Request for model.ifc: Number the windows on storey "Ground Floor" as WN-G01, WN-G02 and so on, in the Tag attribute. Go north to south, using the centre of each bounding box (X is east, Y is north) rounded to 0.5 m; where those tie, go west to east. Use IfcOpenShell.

First a look at what the model holds.

```python
import ifcopenshell
import ifcopenshell.util.element
import ifcopenshell.util.placement

model = ifcopenshell.open("model.ifc")
print(model.schema)
storey = next(s for s in model.by_type("IfcBuildingStorey") if s.Name == "Ground Floor")
windows = [e for e in ifcopenshell.util.element.get_decomposition(storey) if e.is_a("IfcWindow")]
for e in sorted(windows, key=lambda e: e.id()):
    origin = ifcopenshell.util.placement.get_local_placement(e.ObjectPlacement)[:3, 3]
    print(e.id(), e.Tag, e.Name, origin.round(2) + 0.0, sep=" | ")
```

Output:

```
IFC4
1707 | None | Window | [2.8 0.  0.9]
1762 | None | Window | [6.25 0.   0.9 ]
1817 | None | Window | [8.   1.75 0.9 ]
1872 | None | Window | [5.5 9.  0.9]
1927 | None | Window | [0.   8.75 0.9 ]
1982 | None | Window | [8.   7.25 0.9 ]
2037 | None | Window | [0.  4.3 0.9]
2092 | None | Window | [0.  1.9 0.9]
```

```python
import ifcopenshell
import ifcopenshell.geom
import ifcopenshell.util.element
import ifcopenshell.util.shape

model = ifcopenshell.open("model.ifc")
settings = ifcopenshell.geom.settings()
settings.set("use-world-coords", True)


def centre(element):
    shape = ifcopenshell.geom.create_shape(settings, element)
    return ifcopenshell.util.shape.get_bbox_centroid(shape.geometry)


storey = next(s for s in model.by_type("IfcBuildingStorey") if s.Name == "Ground Floor")
windows = [e for e in ifcopenshell.util.element.get_decomposition(storey) if e.is_a("IfcWindow")]

# Insertion points can sit at a corner or the storey origin, so sort by the geometry (in metres).
centres = {e: centre(e) for e in windows}
windows.sort(key=lambda e: (-round(centres[e][1] / 0.5), centres[e][0]))

for i, e in enumerate(windows, start=1):
    number = f"WN-G{i:02d}"
    e.Tag = number
    print(e.id(), number)

model.write("model_edited.ifc")
```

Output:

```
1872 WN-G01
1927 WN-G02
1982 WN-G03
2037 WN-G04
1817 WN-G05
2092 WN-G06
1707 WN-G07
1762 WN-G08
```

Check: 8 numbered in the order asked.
